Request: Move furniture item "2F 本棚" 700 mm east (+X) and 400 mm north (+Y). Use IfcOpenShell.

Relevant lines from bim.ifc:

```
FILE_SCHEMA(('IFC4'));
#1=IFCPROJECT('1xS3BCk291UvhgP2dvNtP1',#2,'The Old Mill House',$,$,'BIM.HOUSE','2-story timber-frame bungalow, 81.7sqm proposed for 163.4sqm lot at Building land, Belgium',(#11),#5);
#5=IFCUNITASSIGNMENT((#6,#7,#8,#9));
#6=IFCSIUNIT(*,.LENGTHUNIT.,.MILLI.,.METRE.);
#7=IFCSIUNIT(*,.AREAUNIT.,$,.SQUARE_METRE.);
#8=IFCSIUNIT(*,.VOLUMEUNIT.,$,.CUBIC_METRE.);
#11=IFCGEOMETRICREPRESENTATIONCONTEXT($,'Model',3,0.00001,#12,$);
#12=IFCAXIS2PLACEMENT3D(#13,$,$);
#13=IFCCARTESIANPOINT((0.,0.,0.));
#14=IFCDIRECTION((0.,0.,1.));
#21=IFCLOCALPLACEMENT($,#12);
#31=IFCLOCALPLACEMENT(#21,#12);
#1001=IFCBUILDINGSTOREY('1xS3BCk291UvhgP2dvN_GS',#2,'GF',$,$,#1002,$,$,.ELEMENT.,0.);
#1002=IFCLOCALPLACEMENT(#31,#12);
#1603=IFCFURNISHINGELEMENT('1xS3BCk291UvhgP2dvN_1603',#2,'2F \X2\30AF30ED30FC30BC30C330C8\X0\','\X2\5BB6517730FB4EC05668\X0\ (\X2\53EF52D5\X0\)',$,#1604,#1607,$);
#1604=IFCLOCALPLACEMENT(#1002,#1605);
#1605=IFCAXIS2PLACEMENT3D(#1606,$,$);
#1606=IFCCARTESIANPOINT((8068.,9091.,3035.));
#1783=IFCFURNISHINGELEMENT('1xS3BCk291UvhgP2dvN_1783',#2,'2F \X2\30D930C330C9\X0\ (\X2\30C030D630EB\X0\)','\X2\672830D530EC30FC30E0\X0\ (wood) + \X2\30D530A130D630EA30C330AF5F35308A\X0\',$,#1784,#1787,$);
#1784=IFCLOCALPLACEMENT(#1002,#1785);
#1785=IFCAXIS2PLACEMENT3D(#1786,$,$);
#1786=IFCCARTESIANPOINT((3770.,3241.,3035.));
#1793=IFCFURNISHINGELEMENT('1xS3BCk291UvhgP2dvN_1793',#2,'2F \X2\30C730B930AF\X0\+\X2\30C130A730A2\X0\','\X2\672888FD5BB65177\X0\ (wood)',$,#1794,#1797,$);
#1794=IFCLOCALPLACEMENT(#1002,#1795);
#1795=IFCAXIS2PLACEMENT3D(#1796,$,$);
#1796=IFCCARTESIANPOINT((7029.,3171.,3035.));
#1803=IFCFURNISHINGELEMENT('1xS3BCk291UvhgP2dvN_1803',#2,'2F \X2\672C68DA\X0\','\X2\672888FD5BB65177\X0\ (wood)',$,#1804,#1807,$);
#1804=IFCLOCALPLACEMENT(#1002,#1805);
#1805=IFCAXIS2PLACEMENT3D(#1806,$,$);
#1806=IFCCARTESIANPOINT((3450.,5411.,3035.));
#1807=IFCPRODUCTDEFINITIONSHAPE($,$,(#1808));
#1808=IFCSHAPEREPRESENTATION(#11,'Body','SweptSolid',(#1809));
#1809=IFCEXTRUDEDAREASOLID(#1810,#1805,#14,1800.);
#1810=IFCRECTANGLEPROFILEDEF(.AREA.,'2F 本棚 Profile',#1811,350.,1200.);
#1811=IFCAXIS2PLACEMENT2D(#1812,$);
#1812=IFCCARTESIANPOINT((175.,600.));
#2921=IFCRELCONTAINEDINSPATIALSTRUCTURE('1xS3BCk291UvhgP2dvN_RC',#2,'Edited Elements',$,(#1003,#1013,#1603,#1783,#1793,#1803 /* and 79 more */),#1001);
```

```python
import ifcopenshell
import ifcopenshell.api.geometry
import ifcopenshell.util.placement
import ifcopenshell.util.unit

model = ifcopenshell.open("bim.ifc")
unit_scale = ifcopenshell.util.unit.calculate_unit_scale(model)

item = model.by_guid("1xS3BCk291UvhgP2dvN_1803")
matrix = ifcopenshell.util.placement.get_local_placement(item.ObjectPlacement)
matrix[0, 3] += 0.7 / unit_scale
matrix[1, 3] += 0.4 / unit_scale
ifcopenshell.api.geometry.edit_object_placement(model, product=item, matrix=matrix, is_si=False)

print(ifcopenshell.util.placement.get_local_placement(item.ObjectPlacement).round(3) + 0.0)

model.write("bim_edited.ifc")
```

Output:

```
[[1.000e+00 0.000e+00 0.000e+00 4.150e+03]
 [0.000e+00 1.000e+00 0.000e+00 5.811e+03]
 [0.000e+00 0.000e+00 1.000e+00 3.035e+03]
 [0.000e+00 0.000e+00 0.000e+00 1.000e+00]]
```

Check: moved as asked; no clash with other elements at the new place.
